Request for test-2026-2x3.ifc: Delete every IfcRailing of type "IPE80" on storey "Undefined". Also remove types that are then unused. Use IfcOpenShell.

First a look at what the model holds.

```python
import ifcopenshell
import ifcopenshell.util.element

model = ifcopenshell.open("test-2026-2x3.ifc")
print(model.schema)
storey = next(s for s in model.by_type("IfcBuildingStorey") if s.Name == "Undefined")
railings = [e for e in ifcopenshell.util.element.get_decomposition(storey) if e.is_a("IfcRailing")]
seen = {}
for e in railings:
    element_type = ifcopenshell.util.element.get_type(e)
    name = element_type.Name if element_type not in (None, e) else None
    seen[name] = seen.get(name, 0) + 1
for name, count in sorted(seen.items(), key=str):
    print(count, "x", name)
```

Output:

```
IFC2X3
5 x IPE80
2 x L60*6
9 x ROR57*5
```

```python
import ifcopenshell
import ifcopenshell.api.root
import ifcopenshell.util.element

model = ifcopenshell.open("test-2026-2x3.ifc")

storey = next(s for s in model.by_type("IfcBuildingStorey") if s.Name == "Undefined")
railings = [e for e in ifcopenshell.util.element.get_decomposition(storey) if e.is_a("IfcRailing")]
targets = [e for e in railings if (t := ifcopenshell.util.element.get_type(e)) not in (None, e) and t.Name == "IPE80"]
types = {ifcopenshell.util.element.get_type(e) for e in targets} - {None, *targets}

for e in targets:
    ifcopenshell.api.root.remove_product(model, product=e)
print(len(targets), "removed")

unused = [t for t in types if not ifcopenshell.util.element.get_types(t)]
for t in unused:
    ifcopenshell.api.root.remove_product(model, product=t)
print(len(unused), "unused types removed")

model.write("test-2026-2x3-out.ifc")
```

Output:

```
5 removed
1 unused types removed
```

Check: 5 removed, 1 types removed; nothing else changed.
